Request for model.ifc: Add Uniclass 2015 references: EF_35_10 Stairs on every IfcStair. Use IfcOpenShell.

First a look at what the model holds.

```python
import ifcopenshell

model = ifcopenshell.open("model.ifc")
print(model.schema)
print("classifications:", [c.Name for c in model.by_type("IfcClassification")])
for ifc_class in ("IfcDoor", "IfcRoof", "IfcStair", "IfcWall", "IfcWindow"):
    print(ifc_class, len(model.by_type(ifc_class)))
```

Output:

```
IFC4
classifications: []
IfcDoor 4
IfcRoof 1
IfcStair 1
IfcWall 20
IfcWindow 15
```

```python
import ifcopenshell
import ifcopenshell.api.classification

model = ifcopenshell.open("model.ifc")

system = ifcopenshell.api.classification.add_classification(model, classification="Uniclass 2015")

codes = {
    "IfcStair": ("EF_35_10", "Stairs"),
}
for ifc_class, (code, name) in codes.items():
    products = model.by_type(ifc_class)
    ifcopenshell.api.classification.add_reference(
        model, products=products, classification=system, identification=code, name=name
    )
    print(code, len(products))

model.write("model_updated.ifc")
```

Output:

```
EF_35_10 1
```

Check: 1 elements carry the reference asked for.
